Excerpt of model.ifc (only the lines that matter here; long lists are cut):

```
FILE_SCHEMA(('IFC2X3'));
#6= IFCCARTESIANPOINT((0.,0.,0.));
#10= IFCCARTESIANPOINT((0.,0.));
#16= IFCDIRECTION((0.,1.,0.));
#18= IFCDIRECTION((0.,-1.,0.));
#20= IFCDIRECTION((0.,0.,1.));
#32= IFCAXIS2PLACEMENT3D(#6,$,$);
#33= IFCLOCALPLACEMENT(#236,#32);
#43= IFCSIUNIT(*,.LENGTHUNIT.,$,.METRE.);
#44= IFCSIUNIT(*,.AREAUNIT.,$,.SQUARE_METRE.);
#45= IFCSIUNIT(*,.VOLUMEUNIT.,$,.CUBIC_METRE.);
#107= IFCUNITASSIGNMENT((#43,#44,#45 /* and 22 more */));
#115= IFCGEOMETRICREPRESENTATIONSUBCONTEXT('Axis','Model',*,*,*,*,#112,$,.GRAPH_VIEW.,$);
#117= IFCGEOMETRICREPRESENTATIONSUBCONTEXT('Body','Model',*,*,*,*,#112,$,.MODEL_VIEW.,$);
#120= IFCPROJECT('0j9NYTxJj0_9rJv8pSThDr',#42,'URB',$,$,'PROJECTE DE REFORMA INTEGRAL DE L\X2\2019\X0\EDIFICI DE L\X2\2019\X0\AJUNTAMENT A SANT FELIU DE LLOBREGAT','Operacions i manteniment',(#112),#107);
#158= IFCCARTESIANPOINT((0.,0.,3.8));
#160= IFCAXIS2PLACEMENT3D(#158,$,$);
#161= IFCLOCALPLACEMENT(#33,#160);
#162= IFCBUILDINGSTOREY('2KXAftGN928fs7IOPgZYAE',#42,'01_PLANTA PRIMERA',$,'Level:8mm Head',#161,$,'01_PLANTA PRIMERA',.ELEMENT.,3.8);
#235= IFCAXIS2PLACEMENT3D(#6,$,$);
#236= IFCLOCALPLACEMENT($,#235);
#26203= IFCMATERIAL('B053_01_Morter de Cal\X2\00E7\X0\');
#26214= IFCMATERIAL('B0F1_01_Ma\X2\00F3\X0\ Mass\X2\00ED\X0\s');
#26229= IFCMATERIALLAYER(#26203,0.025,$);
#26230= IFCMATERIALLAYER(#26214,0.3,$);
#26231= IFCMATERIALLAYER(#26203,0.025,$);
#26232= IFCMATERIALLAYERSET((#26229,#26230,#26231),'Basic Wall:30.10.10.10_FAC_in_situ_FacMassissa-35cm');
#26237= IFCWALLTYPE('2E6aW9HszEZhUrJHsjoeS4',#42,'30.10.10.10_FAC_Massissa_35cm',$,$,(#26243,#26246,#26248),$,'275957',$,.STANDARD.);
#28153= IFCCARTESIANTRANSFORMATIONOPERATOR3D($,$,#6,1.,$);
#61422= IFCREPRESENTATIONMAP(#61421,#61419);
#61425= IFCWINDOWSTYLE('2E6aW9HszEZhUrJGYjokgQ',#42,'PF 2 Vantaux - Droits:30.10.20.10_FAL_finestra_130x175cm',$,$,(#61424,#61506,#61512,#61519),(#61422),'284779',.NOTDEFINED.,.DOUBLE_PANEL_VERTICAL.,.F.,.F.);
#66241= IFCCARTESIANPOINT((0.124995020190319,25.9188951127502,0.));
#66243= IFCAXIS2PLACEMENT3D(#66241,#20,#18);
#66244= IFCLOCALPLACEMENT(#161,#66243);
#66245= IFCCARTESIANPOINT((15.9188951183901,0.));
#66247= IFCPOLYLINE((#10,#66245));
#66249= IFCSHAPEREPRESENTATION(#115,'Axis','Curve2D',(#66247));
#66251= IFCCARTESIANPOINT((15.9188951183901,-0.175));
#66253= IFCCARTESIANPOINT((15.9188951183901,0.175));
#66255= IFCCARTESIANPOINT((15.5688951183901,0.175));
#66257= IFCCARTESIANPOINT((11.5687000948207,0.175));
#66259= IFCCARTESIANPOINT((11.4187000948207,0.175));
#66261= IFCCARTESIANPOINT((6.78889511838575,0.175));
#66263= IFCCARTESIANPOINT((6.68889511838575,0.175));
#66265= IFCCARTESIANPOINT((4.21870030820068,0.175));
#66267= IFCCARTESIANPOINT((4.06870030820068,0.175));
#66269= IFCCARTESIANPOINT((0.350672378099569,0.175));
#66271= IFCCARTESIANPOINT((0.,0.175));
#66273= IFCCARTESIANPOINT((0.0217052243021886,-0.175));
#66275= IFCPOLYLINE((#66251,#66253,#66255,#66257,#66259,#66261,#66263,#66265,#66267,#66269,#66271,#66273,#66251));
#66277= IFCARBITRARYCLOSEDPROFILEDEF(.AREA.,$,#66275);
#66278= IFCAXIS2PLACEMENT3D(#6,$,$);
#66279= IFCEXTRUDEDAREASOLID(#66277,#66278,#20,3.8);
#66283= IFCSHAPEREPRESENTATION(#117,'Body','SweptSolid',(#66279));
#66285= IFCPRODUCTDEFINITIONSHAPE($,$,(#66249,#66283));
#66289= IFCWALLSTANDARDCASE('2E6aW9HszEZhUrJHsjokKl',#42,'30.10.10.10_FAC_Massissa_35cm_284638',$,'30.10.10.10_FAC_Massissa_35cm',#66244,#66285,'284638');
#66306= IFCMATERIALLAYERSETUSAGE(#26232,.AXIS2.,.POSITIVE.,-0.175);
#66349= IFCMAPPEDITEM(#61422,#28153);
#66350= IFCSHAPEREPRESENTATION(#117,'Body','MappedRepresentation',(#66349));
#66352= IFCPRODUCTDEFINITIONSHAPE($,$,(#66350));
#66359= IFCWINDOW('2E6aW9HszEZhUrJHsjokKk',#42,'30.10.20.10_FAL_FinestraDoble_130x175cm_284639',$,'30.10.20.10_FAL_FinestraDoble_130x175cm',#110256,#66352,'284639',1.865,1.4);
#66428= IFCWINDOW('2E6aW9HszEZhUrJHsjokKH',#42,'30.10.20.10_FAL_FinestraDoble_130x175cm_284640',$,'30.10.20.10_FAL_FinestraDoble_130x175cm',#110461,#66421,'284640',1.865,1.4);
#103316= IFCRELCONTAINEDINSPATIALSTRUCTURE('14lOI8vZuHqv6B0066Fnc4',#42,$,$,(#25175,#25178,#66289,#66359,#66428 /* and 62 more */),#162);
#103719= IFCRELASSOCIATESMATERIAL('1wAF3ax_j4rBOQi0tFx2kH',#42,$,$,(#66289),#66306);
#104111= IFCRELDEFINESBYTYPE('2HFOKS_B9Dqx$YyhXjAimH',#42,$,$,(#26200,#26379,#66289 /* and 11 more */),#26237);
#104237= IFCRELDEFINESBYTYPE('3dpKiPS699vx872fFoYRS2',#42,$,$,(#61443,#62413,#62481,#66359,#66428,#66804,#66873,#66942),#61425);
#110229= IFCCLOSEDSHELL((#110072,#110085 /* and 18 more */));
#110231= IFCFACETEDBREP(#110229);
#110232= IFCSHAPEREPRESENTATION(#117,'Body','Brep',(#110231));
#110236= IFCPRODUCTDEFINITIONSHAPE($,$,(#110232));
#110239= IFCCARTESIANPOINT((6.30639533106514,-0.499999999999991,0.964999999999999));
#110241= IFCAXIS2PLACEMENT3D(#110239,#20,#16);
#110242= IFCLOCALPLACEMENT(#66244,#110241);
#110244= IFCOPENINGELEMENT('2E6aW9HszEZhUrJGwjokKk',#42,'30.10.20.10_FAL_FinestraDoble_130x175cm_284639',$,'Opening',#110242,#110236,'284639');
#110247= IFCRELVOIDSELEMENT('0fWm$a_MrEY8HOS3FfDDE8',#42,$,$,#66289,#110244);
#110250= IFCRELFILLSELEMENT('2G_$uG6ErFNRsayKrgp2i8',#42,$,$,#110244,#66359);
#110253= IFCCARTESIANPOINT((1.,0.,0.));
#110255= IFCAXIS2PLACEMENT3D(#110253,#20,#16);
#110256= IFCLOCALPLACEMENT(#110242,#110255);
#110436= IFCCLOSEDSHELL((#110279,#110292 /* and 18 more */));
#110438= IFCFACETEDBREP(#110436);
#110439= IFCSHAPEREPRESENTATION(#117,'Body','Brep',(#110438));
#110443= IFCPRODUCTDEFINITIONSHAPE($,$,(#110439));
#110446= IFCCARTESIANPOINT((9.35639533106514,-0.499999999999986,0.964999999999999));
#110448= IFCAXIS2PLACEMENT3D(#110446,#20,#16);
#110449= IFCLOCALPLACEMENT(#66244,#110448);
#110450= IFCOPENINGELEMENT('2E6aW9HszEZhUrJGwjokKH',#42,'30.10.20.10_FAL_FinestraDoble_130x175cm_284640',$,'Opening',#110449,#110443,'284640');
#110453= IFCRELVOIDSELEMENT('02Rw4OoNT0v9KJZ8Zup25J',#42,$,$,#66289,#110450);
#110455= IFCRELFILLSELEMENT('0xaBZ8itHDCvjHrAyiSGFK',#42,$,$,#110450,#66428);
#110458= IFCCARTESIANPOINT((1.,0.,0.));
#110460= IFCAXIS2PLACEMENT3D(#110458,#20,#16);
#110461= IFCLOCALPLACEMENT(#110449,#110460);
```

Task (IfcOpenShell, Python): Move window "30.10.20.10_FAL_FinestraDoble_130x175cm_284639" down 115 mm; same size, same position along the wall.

```python
import numpy as np
import ifcopenshell
import ifcopenshell.api.geometry
import ifcopenshell.util.placement
import ifcopenshell.util.unit

model = ifcopenshell.open("model.ifc")
unit_scale = ifcopenshell.util.unit.calculate_unit_scale(model)

window = model.by_guid("2E6aW9HszEZhUrJHsjokKk")
opening = window.FillsVoids[0].RelatingOpeningElement
dz = -0.115 / unit_scale

shift = np.array([0.0, 0.0, dz])
# The window is placed relative to its opening, so it follows when the opening moves.
matrix = ifcopenshell.util.placement.get_local_placement(opening.ObjectPlacement)
matrix[:3, 3] += shift
ifcopenshell.api.geometry.edit_object_placement(
    model, product=opening, matrix=matrix, is_si=False, should_transform_children=True
)

print(f"moved by {dz * unit_scale:+.3f} m")

model.write("model_rev.ifc")
```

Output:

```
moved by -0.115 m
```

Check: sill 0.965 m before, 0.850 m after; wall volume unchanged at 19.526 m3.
